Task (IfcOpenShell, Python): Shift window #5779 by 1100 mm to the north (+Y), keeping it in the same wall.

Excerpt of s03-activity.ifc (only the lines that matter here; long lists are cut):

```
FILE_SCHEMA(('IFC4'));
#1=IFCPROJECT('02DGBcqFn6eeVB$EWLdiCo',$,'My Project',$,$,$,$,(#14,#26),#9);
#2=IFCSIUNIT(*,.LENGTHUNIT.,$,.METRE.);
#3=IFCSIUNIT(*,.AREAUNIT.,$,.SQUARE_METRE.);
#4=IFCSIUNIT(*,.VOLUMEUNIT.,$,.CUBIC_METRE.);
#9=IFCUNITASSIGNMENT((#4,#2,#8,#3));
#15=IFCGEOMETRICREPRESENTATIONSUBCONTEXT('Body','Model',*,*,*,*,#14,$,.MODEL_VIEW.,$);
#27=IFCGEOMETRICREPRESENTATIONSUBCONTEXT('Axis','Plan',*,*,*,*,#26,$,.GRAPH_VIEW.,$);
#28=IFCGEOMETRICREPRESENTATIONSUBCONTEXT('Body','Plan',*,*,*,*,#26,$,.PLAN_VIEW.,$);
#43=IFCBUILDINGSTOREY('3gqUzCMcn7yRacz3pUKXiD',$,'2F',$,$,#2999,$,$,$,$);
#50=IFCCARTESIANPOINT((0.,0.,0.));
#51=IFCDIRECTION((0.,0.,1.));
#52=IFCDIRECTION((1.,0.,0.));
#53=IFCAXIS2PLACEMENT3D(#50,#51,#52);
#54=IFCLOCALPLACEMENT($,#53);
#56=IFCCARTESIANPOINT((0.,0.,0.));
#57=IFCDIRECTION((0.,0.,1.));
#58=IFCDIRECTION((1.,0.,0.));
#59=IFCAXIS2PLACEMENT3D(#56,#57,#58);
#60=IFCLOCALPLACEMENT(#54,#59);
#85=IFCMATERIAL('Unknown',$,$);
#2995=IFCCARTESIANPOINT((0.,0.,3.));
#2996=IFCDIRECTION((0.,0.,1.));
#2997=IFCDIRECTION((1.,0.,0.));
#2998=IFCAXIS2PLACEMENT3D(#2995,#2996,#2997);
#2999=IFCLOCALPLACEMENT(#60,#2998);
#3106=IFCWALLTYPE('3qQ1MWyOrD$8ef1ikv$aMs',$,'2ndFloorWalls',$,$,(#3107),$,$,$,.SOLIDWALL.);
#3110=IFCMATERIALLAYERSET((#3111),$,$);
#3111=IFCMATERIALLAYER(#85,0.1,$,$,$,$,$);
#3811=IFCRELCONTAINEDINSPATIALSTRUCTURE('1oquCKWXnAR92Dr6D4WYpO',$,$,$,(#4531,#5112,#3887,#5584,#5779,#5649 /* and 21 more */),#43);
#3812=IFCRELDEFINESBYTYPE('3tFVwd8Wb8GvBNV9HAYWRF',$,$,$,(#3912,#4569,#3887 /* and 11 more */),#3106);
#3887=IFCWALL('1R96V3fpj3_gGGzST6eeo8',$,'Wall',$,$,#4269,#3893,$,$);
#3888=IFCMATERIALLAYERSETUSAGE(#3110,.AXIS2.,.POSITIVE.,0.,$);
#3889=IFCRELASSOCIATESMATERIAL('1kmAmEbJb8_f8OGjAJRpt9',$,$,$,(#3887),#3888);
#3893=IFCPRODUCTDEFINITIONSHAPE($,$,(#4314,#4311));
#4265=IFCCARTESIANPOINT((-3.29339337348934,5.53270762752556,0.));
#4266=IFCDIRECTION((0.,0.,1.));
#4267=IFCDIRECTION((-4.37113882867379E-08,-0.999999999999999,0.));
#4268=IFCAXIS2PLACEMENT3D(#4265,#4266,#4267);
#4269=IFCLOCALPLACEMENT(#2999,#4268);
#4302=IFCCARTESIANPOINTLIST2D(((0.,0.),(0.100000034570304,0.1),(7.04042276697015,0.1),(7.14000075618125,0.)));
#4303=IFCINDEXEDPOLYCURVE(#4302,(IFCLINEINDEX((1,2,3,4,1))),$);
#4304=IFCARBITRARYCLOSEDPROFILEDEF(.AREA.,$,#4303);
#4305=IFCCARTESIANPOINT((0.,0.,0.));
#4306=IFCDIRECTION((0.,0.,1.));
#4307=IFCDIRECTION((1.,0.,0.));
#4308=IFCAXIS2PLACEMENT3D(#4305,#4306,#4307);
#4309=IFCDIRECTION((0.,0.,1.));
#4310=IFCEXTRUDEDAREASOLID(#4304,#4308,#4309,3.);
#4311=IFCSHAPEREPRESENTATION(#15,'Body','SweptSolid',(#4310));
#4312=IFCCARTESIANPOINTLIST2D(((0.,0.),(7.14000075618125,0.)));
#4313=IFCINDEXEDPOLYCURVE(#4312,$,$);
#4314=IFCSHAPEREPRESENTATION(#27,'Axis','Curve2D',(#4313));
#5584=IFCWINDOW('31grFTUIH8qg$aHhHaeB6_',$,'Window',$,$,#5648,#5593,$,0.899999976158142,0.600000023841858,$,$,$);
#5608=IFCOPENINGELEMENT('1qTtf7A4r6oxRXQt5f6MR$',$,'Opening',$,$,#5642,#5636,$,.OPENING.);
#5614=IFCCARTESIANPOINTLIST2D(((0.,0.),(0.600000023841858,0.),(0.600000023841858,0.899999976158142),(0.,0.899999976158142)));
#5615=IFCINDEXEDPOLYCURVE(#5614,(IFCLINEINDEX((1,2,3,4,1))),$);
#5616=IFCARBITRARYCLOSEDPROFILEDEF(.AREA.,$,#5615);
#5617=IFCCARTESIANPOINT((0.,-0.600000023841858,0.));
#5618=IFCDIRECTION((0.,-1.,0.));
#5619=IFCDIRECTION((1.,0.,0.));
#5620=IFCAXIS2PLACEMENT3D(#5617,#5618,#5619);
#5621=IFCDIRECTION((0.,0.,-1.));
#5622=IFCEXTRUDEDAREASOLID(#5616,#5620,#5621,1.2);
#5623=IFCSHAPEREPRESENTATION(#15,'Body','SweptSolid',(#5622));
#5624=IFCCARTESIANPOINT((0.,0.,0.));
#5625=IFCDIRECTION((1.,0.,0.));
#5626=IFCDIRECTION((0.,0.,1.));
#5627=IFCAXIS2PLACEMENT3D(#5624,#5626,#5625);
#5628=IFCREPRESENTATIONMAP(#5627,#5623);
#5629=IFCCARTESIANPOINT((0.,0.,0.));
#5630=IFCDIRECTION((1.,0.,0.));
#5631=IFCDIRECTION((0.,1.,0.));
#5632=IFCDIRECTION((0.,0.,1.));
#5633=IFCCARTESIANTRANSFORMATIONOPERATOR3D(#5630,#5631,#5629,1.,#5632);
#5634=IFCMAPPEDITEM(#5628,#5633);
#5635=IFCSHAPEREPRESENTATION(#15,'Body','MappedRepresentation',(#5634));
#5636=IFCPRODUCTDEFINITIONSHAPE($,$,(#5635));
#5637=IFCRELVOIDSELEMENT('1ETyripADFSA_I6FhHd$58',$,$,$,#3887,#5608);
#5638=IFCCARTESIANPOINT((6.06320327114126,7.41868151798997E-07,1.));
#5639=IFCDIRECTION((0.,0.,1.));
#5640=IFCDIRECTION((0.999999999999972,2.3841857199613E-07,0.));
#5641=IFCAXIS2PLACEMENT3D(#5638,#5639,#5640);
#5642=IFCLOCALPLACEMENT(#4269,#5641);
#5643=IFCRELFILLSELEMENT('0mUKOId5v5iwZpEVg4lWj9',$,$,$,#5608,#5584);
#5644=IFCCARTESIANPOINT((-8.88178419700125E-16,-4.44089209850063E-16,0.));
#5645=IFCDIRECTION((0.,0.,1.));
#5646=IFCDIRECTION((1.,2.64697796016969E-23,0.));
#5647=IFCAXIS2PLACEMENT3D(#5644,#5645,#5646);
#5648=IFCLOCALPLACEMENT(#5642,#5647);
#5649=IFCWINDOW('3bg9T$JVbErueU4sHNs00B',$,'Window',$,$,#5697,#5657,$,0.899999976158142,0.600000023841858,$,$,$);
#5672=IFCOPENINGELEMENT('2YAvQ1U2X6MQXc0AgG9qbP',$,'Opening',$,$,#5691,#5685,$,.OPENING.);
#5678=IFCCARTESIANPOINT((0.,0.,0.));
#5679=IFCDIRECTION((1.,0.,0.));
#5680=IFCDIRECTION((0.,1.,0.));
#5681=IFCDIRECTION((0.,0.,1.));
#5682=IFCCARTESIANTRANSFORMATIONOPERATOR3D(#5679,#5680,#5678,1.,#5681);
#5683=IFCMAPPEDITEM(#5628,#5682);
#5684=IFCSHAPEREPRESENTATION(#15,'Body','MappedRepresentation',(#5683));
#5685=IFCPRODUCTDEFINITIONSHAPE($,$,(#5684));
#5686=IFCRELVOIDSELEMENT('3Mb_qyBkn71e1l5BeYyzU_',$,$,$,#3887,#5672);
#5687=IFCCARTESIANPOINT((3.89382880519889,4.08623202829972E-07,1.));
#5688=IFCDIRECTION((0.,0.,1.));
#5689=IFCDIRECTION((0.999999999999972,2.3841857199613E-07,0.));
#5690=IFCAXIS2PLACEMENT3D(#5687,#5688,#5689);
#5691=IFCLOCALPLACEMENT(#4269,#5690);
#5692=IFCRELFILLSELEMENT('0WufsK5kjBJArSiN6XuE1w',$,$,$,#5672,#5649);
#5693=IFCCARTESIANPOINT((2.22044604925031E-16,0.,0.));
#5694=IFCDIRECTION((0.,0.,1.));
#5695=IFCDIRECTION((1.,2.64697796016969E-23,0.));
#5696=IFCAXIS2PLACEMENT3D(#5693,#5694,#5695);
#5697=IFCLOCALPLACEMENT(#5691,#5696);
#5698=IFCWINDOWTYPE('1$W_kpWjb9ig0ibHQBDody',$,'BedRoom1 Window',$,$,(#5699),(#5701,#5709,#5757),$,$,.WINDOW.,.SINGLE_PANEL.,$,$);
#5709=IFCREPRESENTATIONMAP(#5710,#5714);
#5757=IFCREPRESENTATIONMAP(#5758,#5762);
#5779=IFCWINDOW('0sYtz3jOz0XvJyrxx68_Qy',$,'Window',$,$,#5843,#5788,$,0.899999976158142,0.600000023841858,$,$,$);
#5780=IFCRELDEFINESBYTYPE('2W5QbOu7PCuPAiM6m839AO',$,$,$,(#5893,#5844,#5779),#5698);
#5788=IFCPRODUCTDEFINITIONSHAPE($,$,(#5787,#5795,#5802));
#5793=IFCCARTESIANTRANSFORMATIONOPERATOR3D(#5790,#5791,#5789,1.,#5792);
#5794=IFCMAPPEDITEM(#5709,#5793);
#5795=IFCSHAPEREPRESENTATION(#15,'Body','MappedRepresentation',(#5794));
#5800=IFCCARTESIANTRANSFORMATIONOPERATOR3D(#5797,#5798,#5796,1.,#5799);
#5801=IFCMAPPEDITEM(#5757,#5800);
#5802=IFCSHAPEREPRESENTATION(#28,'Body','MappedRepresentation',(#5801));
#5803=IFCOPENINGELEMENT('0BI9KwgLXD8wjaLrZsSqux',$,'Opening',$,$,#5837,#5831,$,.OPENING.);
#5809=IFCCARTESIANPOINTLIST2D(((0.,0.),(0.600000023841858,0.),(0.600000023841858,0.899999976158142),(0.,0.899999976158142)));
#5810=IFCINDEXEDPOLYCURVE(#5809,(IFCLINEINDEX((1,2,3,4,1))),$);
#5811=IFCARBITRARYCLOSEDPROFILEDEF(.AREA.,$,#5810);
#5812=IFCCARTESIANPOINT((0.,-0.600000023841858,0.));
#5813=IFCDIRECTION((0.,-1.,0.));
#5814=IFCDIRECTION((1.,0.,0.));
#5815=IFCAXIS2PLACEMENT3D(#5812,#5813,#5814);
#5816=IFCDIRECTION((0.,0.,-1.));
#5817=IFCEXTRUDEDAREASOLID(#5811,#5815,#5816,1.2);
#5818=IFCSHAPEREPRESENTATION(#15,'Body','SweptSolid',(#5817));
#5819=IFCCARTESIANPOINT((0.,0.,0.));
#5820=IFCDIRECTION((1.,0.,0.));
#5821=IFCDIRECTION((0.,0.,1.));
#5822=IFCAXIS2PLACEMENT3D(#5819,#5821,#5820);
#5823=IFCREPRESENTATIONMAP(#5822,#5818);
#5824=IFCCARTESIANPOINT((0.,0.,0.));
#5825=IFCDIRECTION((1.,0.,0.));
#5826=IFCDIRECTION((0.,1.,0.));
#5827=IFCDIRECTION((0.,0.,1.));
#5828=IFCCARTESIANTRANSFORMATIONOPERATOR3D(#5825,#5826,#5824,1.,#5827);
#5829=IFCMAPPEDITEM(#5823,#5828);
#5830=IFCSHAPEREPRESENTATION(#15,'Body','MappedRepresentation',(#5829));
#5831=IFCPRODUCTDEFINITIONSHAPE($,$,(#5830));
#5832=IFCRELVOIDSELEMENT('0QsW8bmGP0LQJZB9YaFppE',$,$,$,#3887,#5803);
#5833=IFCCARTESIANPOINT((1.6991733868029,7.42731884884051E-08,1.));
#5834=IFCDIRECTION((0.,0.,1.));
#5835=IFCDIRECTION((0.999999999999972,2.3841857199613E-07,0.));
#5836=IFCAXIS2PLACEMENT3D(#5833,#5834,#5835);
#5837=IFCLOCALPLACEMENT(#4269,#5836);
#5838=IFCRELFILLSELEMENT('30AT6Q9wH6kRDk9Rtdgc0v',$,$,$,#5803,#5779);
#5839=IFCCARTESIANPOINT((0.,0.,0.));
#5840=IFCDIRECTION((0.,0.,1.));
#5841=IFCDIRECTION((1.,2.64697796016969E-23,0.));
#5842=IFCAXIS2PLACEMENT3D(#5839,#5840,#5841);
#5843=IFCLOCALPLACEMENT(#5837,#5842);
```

```python
import ifcopenshell
import ifcopenshell.api.geometry
import ifcopenshell.util.placement
import ifcopenshell.util.unit

model = ifcopenshell.open("s03-activity.ifc")
unit_scale = ifcopenshell.util.unit.calculate_unit_scale(model)

window = model.by_guid("0sYtz3jOz0XvJyrxx68_Qy")
opening = window.FillsVoids[0].RelatingOpeningElement
wall = opening.VoidsElements[0].RelatingBuildingElement

wall_matrix = ifcopenshell.util.placement.get_local_placement(wall.ObjectPlacement)
shift = wall_matrix[:3, 0] * -1.1 / unit_scale
before = ifcopenshell.util.placement.get_local_placement(window.ObjectPlacement)[:3, 3].copy()

# The window is placed relative to its opening, so it follows when the opening moves.
matrix = ifcopenshell.util.placement.get_local_placement(opening.ObjectPlacement)
matrix[:3, 3] += shift
ifcopenshell.api.geometry.edit_object_placement(
    model, product=opening, matrix=matrix, is_si=False, should_transform_children=True
)

after = ifcopenshell.util.placement.get_local_placement(window.ObjectPlacement)[:3, 3]
print("window moved by", (after - before).round(3) + 0.0)

model.write("s03-activity_updated.ifc")
```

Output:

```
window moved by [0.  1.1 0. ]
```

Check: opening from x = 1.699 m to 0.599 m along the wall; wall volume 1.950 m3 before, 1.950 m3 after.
